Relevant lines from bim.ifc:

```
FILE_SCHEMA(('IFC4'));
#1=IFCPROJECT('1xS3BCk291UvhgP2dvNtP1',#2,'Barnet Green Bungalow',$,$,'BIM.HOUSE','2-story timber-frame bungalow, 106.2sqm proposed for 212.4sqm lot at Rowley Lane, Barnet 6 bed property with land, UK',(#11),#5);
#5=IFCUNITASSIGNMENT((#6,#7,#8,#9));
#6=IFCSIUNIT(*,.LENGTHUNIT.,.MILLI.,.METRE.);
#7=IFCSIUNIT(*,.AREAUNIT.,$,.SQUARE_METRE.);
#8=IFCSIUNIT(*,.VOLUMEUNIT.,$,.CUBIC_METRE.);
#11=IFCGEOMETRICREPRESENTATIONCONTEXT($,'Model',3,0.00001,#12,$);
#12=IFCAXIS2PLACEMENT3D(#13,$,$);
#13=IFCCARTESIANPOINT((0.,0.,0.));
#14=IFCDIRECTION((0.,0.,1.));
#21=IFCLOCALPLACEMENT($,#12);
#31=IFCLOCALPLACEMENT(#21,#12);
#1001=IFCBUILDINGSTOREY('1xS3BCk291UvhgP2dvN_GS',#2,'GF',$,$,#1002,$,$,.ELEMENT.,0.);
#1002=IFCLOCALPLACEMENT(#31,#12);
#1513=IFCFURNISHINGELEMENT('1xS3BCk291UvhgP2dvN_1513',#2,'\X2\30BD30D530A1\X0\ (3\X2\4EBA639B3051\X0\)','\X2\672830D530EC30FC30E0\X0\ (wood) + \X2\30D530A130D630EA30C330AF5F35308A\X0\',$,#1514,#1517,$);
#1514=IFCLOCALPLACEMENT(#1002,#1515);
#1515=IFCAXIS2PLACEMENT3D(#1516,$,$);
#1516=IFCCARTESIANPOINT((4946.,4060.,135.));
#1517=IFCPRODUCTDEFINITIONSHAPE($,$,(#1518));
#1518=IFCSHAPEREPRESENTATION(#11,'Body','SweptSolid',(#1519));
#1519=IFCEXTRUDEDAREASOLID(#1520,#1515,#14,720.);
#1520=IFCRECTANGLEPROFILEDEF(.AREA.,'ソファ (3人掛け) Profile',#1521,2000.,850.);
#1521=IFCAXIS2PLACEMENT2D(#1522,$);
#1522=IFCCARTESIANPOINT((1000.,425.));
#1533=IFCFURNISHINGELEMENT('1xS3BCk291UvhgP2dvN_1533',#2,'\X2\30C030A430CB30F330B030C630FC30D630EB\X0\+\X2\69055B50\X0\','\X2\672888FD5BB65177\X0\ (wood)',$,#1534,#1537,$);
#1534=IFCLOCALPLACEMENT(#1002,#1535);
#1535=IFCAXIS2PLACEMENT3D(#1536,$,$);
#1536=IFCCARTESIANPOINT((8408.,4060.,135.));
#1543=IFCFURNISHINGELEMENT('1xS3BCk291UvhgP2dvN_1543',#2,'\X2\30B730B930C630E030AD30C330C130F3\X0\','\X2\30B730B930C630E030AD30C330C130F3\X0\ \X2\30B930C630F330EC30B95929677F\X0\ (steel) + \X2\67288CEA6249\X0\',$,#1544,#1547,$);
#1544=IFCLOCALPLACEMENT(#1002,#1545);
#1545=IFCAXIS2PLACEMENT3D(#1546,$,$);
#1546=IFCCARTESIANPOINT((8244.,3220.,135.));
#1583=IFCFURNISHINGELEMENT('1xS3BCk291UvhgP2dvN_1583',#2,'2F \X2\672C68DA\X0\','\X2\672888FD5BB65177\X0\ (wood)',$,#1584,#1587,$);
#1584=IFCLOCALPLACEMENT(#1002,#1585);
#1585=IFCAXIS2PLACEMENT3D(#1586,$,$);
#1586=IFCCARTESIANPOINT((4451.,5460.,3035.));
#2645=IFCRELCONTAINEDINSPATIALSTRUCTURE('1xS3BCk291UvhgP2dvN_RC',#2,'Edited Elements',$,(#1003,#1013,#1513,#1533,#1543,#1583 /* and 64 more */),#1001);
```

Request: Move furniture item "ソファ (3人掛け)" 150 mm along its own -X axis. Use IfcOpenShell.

```python
import ifcopenshell
import ifcopenshell.api.geometry
import ifcopenshell.util.placement

model = ifcopenshell.open("bim.ifc")

item = model.by_guid("1xS3BCk291UvhgP2dvN_1513")
matrix = ifcopenshell.util.placement.get_local_placement(item.ObjectPlacement)
matrix[:3, 3] -= matrix[:3, 0] * 150.0
ifcopenshell.api.geometry.edit_object_placement(model, product=item, matrix=matrix, is_si=False)

print(ifcopenshell.util.placement.get_local_placement(item.ObjectPlacement).round(3) + 0.0)

model.write("bim_edited.ifc")
```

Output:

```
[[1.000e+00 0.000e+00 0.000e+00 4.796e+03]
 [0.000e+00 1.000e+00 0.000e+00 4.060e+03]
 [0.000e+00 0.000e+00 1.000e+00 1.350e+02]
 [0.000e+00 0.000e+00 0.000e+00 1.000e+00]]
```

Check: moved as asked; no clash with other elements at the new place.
